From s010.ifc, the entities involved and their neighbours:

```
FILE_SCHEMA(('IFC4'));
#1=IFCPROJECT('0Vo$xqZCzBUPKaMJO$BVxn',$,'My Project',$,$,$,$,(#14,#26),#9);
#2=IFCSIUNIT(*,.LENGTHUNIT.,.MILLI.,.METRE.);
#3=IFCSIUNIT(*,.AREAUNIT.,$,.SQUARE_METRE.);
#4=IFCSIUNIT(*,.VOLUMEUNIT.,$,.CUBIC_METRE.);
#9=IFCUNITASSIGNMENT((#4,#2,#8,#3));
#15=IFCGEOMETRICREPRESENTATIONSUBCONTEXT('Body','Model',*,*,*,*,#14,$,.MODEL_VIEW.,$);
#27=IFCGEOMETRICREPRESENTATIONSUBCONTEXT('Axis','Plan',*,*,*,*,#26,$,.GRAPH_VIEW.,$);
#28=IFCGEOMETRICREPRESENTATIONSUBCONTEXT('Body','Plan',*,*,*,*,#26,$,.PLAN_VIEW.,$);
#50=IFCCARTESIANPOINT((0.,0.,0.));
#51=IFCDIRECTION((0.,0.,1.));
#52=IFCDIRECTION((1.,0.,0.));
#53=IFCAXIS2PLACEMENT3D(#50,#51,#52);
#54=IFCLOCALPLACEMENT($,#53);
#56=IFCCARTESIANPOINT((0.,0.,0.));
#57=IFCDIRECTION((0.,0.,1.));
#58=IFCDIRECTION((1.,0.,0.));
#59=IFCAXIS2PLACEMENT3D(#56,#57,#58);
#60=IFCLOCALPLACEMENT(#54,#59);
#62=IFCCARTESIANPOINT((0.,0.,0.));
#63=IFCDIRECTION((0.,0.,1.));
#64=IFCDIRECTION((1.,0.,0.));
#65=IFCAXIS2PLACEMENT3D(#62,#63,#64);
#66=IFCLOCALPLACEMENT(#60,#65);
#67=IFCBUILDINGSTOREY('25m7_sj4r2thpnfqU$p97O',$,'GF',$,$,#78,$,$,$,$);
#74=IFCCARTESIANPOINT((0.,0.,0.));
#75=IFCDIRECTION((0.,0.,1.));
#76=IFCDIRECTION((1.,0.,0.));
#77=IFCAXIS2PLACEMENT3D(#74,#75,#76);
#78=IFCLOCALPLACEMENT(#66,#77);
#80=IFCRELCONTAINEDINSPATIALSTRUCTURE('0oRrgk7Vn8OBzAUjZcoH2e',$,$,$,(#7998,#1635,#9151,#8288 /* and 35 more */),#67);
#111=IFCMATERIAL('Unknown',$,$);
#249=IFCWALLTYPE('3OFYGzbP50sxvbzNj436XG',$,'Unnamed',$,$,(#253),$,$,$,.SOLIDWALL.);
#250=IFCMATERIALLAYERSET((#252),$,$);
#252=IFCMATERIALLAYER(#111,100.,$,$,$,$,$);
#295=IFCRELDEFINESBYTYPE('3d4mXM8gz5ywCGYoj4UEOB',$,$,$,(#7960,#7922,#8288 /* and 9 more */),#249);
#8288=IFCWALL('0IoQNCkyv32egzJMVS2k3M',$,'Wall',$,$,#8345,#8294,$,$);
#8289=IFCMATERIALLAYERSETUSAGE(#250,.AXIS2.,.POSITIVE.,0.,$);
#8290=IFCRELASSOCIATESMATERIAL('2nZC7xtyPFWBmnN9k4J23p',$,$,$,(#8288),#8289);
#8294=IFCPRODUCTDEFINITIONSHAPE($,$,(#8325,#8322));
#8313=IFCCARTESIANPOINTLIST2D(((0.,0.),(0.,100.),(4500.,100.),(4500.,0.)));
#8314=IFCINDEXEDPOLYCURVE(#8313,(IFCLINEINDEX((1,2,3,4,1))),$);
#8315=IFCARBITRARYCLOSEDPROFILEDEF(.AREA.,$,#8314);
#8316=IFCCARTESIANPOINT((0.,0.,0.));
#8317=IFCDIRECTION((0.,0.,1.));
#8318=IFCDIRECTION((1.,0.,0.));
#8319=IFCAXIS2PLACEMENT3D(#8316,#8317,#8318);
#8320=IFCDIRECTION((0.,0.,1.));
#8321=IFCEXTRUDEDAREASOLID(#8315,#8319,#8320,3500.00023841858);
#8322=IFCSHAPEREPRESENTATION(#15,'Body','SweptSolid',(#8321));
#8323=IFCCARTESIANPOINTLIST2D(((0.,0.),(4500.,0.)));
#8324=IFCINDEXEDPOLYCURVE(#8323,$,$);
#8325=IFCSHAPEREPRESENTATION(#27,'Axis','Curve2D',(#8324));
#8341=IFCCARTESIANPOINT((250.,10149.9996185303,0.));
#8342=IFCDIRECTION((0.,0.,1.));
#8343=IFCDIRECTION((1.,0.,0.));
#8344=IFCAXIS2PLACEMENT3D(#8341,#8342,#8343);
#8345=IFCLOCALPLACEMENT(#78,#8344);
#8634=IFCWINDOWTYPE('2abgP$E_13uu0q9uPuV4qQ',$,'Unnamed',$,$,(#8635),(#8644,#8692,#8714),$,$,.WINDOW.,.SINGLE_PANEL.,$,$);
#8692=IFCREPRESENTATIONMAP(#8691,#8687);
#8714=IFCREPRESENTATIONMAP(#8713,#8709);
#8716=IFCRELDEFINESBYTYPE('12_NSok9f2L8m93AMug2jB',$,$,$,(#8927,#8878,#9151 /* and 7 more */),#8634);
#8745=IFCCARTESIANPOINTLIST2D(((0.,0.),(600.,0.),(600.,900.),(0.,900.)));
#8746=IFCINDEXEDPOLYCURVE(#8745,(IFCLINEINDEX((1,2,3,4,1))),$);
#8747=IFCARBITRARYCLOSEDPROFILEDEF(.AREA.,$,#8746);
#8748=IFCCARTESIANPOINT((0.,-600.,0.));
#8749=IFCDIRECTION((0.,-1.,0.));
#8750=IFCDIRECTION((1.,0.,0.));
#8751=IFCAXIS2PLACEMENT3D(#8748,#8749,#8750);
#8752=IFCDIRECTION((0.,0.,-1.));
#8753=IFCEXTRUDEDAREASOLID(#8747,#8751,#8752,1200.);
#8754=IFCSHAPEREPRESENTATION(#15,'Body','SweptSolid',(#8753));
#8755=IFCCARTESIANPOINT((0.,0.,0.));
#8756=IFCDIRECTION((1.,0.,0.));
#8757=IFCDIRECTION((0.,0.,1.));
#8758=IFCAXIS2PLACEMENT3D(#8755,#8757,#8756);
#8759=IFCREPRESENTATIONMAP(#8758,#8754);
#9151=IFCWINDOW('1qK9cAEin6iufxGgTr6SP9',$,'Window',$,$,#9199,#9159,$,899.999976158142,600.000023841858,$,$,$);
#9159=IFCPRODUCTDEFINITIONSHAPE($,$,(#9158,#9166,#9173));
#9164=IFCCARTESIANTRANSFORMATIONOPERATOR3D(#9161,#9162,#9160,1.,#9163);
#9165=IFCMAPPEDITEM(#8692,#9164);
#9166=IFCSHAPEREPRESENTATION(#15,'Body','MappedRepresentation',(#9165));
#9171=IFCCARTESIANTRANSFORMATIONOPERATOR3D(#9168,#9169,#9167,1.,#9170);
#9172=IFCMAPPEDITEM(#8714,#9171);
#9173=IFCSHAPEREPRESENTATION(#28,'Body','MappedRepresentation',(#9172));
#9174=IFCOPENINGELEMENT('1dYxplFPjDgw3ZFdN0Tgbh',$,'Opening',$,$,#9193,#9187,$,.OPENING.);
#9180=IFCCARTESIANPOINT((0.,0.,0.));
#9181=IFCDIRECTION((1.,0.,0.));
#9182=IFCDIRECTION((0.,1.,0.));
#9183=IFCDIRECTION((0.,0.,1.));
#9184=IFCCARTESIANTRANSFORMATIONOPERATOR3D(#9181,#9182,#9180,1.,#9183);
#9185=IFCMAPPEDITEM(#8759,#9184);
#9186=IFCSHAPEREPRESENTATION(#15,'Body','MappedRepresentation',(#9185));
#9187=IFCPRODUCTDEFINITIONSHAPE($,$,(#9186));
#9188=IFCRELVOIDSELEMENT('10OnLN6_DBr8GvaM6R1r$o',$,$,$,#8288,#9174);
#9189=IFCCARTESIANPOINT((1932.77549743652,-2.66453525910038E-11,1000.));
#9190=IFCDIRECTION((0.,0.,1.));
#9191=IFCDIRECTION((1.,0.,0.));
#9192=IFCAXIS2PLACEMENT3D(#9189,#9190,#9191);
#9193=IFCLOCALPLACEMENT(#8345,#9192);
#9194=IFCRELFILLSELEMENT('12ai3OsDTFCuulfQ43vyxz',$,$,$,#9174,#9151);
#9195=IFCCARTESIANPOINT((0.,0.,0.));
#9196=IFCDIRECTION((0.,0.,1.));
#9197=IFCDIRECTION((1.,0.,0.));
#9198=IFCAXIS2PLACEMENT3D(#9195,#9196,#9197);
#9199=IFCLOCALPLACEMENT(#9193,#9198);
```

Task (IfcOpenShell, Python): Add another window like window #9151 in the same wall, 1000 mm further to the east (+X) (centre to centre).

```python
import ifcopenshell
import ifcopenshell.api.feature
import ifcopenshell.api.geometry
import ifcopenshell.api.root
import ifcopenshell.geom
import ifcopenshell.util.element
import ifcopenshell.util.placement
import ifcopenshell.util.shape

model = ifcopenshell.open("s010.ifc")
settings = ifcopenshell.geom.settings()


def volume(element):
    """Net volume in cubic metres, openings subtracted."""
    shape = ifcopenshell.geom.create_shape(settings, element)
    return ifcopenshell.util.shape.get_volume(shape.geometry)


window = model.by_guid("1qK9cAEin6iufxGgTr6SP9")
opening = window.FillsVoids[0].RelatingOpeningElement
wall = opening.VoidsElements[0].RelatingBuildingElement
before = volume(wall)
shift = ifcopenshell.util.placement.get_local_placement(wall.ObjectPlacement)[:3, 0] * 1000.0

# copy_class copies the void relationship, type, container and properties, but no geometry.
new_opening = ifcopenshell.api.root.copy_class(model, product=opening)
new_opening.Representation = ifcopenshell.util.element.copy_deep(
    model, opening.Representation, exclude=["IfcGeometricRepresentationContext", "IfcRepresentationMap"]
)
new_window = ifcopenshell.api.root.copy_class(model, product=window)
new_window.Representation = ifcopenshell.util.element.copy_deep(
    model, window.Representation, exclude=["IfcGeometricRepresentationContext", "IfcRepresentationMap"]
)
ifcopenshell.api.feature.add_filling(model, opening=new_opening, element=new_window)

for old, new in ((opening, new_opening), (window, new_window)):
    matrix = ifcopenshell.util.placement.get_local_placement(old.ObjectPlacement)
    matrix[:3, 3] += shift
    ifcopenshell.api.geometry.edit_object_placement(model, product=new, matrix=matrix, is_si=False)

after = volume(wall)

print(f"wall volume {before:.3f} -> {after:.3f} m3")

model.write("s010_updated.ifc")
```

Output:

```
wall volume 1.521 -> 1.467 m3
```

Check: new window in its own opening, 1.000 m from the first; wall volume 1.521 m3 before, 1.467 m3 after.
